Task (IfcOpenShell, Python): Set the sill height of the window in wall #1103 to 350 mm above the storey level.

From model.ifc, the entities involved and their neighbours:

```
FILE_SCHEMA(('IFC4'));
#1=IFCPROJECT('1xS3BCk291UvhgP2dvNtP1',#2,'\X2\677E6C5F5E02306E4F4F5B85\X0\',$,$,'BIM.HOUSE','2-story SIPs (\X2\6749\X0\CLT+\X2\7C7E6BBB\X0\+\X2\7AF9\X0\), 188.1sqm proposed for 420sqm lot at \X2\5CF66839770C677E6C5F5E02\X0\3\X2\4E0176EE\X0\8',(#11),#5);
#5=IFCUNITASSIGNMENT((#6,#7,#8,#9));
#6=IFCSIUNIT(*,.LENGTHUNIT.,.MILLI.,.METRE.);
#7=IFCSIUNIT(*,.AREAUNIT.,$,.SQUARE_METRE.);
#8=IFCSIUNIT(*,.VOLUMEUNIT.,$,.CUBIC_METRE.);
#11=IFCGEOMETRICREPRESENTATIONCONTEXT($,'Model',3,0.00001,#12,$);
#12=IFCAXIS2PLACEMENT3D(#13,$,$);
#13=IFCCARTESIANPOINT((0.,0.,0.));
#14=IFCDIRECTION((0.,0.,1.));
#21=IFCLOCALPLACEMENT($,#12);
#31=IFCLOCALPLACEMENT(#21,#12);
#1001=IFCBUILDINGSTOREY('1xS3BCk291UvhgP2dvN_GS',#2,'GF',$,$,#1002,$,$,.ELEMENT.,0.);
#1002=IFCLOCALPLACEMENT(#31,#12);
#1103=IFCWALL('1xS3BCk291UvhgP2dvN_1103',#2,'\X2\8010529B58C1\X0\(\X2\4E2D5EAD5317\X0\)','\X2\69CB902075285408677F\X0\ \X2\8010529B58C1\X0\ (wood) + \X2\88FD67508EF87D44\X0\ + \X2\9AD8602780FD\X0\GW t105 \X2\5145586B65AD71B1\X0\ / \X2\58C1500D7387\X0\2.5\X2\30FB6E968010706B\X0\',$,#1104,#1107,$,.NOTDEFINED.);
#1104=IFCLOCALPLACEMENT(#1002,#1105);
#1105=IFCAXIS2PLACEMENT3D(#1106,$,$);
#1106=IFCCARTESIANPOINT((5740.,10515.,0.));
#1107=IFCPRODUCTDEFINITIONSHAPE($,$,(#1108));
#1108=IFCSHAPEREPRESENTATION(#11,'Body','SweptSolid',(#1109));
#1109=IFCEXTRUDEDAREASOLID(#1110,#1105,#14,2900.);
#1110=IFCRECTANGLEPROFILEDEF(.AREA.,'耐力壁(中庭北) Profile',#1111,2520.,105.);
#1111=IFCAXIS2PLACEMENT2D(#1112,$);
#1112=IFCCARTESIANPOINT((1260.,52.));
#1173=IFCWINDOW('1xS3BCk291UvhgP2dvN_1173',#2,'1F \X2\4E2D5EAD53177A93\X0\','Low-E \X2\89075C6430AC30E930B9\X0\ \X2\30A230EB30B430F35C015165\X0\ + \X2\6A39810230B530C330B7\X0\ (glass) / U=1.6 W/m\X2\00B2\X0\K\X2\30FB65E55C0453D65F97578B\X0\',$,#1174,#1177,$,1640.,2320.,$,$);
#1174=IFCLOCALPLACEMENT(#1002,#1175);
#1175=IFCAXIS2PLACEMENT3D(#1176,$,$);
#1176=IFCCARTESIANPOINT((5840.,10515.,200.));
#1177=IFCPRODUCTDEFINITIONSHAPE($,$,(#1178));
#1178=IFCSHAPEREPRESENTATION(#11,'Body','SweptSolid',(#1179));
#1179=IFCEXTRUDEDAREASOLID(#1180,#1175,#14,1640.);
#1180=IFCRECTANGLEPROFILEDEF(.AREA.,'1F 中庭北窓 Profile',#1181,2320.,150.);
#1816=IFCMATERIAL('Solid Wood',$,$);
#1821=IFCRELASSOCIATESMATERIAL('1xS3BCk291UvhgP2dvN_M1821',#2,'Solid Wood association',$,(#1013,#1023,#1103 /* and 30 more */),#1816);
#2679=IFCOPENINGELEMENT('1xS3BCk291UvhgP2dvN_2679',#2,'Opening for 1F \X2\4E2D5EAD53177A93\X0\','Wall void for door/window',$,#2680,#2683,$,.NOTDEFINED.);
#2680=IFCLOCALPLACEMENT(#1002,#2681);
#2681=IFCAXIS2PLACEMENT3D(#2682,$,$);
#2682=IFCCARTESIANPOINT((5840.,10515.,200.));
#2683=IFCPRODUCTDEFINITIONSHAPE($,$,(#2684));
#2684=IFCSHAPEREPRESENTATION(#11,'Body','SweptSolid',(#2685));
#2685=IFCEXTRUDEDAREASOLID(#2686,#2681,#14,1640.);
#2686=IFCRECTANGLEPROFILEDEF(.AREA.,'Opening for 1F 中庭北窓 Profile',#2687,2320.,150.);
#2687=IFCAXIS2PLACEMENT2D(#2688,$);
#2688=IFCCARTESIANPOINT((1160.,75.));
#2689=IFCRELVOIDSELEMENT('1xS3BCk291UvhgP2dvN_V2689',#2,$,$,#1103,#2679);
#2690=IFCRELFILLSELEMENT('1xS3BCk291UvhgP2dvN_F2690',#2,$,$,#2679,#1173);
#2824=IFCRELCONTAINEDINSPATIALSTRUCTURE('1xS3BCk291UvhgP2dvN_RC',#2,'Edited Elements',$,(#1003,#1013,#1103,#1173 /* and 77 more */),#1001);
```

```python
import numpy as np
import ifcopenshell
import ifcopenshell.api.geometry
import ifcopenshell.geom
import ifcopenshell.util.element
import ifcopenshell.util.placement
import ifcopenshell.util.shape
import ifcopenshell.util.unit

model = ifcopenshell.open("model.ifc")
unit_scale = ifcopenshell.util.unit.calculate_unit_scale(model)

window = model.by_id(1173)
opening = window.FillsVoids[0].RelatingOpeningElement
storey = ifcopenshell.util.element.get_container(window, ifc_class="IfcBuildingStorey")
level = ifcopenshell.util.placement.get_local_placement(storey.ObjectPlacement)[2, 3]

# The opening's origin need not be at the sill, so measure its lowest point.
shape = ifcopenshell.geom.create_shape(ifcopenshell.geom.settings(), opening)
bottom = ifcopenshell.util.shape.get_shape_bottom_elevation(shape, shape.geometry) / unit_scale
dz = level + 350.0 - bottom

shift = np.array([0.0, 0.0, dz])
# The window is not placed relative to its opening, so move both.
for product in (opening, window):
    matrix = ifcopenshell.util.placement.get_local_placement(product.ObjectPlacement)
    matrix[:3, 3] += shift
    ifcopenshell.api.geometry.edit_object_placement(model, product=product, matrix=matrix, is_si=False)

print(f"moved by {dz * unit_scale:+.3f} m")

model.write("model_edited.ifc")
```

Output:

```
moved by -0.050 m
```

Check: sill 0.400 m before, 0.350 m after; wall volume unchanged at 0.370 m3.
